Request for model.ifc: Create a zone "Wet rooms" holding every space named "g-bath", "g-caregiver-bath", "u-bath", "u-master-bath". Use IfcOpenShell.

First a look at what the model holds.

```python
import ifcopenshell

model = ifcopenshell.open("model.ifc")
print(model.schema)
seen = {}
for space in model.by_type("IfcSpace"):
    seen[space.LongName] = seen.get(space.LongName, 0) + 1
for name, count in sorted(seen.items(), key=str):
    print(count, "x", name)
print("zones:", [z.Name for z in model.by_type("IfcZone")][:20])
```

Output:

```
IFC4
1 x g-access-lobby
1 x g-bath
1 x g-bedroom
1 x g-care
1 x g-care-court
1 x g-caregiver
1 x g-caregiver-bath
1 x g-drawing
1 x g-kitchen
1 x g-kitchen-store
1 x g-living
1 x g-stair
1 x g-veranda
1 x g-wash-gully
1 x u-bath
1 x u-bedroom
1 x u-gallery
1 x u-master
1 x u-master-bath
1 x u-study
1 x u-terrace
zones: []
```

```python
import ifcopenshell
import ifcopenshell.api.group
import ifcopenshell.api.root

model = ifcopenshell.open("model.ifc")

names = {"g-bath", "g-caregiver-bath", "u-bath", "u-master-bath"}
spaces = [s for s in model.by_type("IfcSpace") if s.LongName in names]

zone = ifcopenshell.api.root.create_entity(model, ifc_class="IfcZone", name="Wet rooms")
ifcopenshell.api.group.assign_group(model, products=spaces, group=zone)
print(len(spaces), "spaces in", zone.Name)

model.write("model_v2.ifc")
```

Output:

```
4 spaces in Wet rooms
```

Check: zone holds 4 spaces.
